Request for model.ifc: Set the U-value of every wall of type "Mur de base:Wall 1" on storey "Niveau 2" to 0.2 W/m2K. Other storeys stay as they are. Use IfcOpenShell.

First a look at what the model holds.

```python
import ifcopenshell
import ifcopenshell.util.element

model = ifcopenshell.open("model.ifc")
print(model.schema)
storey = next(s for s in model.by_type("IfcBuildingStorey") if s.Name == "Niveau 2")
walls = [e for e in ifcopenshell.util.element.get_decomposition(storey) if e.is_a("IfcWall")]
seen = {}
for e in walls:
    element_type = ifcopenshell.util.element.get_type(e)
    key = (element_type.Name if element_type != e and element_type else None, ifcopenshell.util.element.get_pset(e, "Pset_WallCommon", "ThermalTransmittance"))
    seen[key] = seen.get(key, 0) + 1
for (name, value), count in sorted(seen.items(), key=str):
    print(count, "x", name, "|", value)
```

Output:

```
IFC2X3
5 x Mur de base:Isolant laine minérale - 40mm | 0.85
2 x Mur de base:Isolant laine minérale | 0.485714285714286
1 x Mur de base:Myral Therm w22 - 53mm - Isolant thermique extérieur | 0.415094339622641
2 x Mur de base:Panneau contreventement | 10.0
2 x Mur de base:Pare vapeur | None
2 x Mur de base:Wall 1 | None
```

```python
import ifcopenshell
import ifcopenshell.api.pset
import ifcopenshell.util.element

model = ifcopenshell.open("model.ifc")

storey = next(s for s in model.by_type("IfcBuildingStorey") if s.Name == "Niveau 2")
walls = [e for e in ifcopenshell.util.element.get_decomposition(storey) if e.is_a("IfcWall")]

count = 0
for e in walls:
    element_type = ifcopenshell.util.element.get_type(e)
    if element_type in (None, e) or element_type.Name != "Mur de base:Wall 1":
        continue
    # add_pset returns the element's existing set when there is one.
    pset = ifcopenshell.api.pset.add_pset(model, product=e, name="Pset_WallCommon")
    ifcopenshell.api.pset.edit_pset(model, pset=pset, properties={"ThermalTransmittance": 0.2})
    count += 1

print(count, "walls updated")

model.write("model_edited.ifc")
```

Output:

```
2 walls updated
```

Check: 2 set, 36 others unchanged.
